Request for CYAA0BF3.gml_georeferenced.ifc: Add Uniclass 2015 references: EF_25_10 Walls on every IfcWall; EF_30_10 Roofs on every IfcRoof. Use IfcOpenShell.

First a look at what the model holds.

```python
import ifcopenshell

model = ifcopenshell.open("CYAA0BF3.gml_georeferenced.ifc")
print(model.schema)
print("classifications:", [c.Name for c in model.by_type("IfcClassification")])
for ifc_class in ("IfcDoor", "IfcRoof", "IfcStair", "IfcWall", "IfcWindow"):
    print(ifc_class, len(model.by_type(ifc_class)))
```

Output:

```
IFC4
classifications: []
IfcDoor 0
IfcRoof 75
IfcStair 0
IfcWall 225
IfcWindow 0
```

```python
import ifcopenshell
import ifcopenshell.api.classification

model = ifcopenshell.open("CYAA0BF3.gml_georeferenced.ifc")

system = ifcopenshell.api.classification.add_classification(model, classification="Uniclass 2015")

codes = {
    "IfcWall": ("EF_25_10", "Walls"),
    "IfcRoof": ("EF_30_10", "Roofs"),
}
for ifc_class, (code, name) in codes.items():
    products = model.by_type(ifc_class)
    ifcopenshell.api.classification.add_reference(
        model, products=products, classification=system, identification=code, name=name
    )
    print(code, len(products))

model.write("CYAA0BF3.gml_georeferenced_v2.ifc")
```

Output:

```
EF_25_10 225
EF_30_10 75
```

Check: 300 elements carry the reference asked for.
